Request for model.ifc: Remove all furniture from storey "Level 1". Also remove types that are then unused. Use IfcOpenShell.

First a look at what the model holds.

```python
import ifcopenshell
import ifcopenshell.util.element

model = ifcopenshell.open("model.ifc")
print(model.schema)
storey = next(s for s in model.by_type("IfcBuildingStorey") if s.Name == "Level 1")
furniture = [e for e in ifcopenshell.util.element.get_decomposition(storey) if e.is_a("IfcFurnishingElement")]
seen = {}
for e in furniture:
    element_type = ifcopenshell.util.element.get_type(e)
    name = element_type.Name if element_type not in (None, e) else None
    seen[name] = seen.get(name, 0) + 1
for name, count in sorted(seen.items(), key=str):
    print(count, "x", name)
```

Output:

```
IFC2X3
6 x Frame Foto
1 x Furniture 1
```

```python
import ifcopenshell
import ifcopenshell.api.root
import ifcopenshell.util.element

model = ifcopenshell.open("model.ifc")

storey = next(s for s in model.by_type("IfcBuildingStorey") if s.Name == "Level 1")
furniture = [e for e in ifcopenshell.util.element.get_decomposition(storey) if e.is_a("IfcFurnishingElement")]
types = {ifcopenshell.util.element.get_type(e) for e in furniture} - {None, *furniture}

for e in furniture:
    ifcopenshell.api.root.remove_product(model, product=e)
print(len(furniture), "removed")

unused = [t for t in types if not ifcopenshell.util.element.get_types(t)]
for t in unused:
    ifcopenshell.api.root.remove_product(model, product=t)
print(len(unused), "unused types removed")

model.write("model_edited.ifc")
```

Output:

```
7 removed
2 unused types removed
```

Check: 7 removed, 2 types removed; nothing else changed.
